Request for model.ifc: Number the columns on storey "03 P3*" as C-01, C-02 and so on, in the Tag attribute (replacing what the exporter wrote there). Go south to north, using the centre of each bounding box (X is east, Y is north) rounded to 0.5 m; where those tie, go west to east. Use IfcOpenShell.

First a look at what the model holds.

```python
import ifcopenshell
import ifcopenshell.util.element
import ifcopenshell.util.placement

model = ifcopenshell.open("model.ifc")
print(model.schema)
storey = next(s for s in model.by_type("IfcBuildingStorey") if s.Name == "03 P3*")
columns = [e for e in ifcopenshell.util.element.get_decomposition(storey) if e.is_a("IfcColumn")]
for e in sorted(columns, key=lambda e: e.id()):
    origin = ifcopenshell.util.placement.get_local_placement(e.ObjectPlacement)[:3, 3]
    print(e.id(), e.Tag, e.Name, origin.round(2) + 0.0, sep=" | ")
```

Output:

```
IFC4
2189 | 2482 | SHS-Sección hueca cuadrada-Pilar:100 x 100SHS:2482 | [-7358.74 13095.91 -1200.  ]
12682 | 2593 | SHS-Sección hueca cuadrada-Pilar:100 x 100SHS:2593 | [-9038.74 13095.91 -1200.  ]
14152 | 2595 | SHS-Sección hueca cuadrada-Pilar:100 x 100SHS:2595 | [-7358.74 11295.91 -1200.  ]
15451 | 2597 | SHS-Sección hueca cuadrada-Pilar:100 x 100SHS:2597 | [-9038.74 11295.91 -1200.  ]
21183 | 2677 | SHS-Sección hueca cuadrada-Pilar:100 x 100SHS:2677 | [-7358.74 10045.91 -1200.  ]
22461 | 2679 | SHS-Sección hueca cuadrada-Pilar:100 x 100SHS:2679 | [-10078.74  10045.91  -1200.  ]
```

```python
import ifcopenshell
import ifcopenshell.geom
import ifcopenshell.util.element
import ifcopenshell.util.shape

model = ifcopenshell.open("model.ifc")
settings = ifcopenshell.geom.settings()
settings.set("use-world-coords", True)


def centre(element):
    shape = ifcopenshell.geom.create_shape(settings, element)
    return ifcopenshell.util.shape.get_bbox_centroid(shape.geometry)


storey = next(s for s in model.by_type("IfcBuildingStorey") if s.Name == "03 P3*")
columns = [e for e in ifcopenshell.util.element.get_decomposition(storey) if e.is_a("IfcColumn")]

# Insertion points can sit at a corner or the storey origin, so sort by the geometry (in metres).
centres = {e: centre(e) for e in columns}
columns.sort(key=lambda e: (round(centres[e][1] / 0.5), centres[e][0]))

for i, e in enumerate(columns, start=1):
    number = f"C-{i:02d}"
    e.Tag = number
    print(e.id(), number)

model.write("model_edited.ifc")
```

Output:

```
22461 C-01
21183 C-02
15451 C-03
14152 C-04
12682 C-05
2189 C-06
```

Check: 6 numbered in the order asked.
